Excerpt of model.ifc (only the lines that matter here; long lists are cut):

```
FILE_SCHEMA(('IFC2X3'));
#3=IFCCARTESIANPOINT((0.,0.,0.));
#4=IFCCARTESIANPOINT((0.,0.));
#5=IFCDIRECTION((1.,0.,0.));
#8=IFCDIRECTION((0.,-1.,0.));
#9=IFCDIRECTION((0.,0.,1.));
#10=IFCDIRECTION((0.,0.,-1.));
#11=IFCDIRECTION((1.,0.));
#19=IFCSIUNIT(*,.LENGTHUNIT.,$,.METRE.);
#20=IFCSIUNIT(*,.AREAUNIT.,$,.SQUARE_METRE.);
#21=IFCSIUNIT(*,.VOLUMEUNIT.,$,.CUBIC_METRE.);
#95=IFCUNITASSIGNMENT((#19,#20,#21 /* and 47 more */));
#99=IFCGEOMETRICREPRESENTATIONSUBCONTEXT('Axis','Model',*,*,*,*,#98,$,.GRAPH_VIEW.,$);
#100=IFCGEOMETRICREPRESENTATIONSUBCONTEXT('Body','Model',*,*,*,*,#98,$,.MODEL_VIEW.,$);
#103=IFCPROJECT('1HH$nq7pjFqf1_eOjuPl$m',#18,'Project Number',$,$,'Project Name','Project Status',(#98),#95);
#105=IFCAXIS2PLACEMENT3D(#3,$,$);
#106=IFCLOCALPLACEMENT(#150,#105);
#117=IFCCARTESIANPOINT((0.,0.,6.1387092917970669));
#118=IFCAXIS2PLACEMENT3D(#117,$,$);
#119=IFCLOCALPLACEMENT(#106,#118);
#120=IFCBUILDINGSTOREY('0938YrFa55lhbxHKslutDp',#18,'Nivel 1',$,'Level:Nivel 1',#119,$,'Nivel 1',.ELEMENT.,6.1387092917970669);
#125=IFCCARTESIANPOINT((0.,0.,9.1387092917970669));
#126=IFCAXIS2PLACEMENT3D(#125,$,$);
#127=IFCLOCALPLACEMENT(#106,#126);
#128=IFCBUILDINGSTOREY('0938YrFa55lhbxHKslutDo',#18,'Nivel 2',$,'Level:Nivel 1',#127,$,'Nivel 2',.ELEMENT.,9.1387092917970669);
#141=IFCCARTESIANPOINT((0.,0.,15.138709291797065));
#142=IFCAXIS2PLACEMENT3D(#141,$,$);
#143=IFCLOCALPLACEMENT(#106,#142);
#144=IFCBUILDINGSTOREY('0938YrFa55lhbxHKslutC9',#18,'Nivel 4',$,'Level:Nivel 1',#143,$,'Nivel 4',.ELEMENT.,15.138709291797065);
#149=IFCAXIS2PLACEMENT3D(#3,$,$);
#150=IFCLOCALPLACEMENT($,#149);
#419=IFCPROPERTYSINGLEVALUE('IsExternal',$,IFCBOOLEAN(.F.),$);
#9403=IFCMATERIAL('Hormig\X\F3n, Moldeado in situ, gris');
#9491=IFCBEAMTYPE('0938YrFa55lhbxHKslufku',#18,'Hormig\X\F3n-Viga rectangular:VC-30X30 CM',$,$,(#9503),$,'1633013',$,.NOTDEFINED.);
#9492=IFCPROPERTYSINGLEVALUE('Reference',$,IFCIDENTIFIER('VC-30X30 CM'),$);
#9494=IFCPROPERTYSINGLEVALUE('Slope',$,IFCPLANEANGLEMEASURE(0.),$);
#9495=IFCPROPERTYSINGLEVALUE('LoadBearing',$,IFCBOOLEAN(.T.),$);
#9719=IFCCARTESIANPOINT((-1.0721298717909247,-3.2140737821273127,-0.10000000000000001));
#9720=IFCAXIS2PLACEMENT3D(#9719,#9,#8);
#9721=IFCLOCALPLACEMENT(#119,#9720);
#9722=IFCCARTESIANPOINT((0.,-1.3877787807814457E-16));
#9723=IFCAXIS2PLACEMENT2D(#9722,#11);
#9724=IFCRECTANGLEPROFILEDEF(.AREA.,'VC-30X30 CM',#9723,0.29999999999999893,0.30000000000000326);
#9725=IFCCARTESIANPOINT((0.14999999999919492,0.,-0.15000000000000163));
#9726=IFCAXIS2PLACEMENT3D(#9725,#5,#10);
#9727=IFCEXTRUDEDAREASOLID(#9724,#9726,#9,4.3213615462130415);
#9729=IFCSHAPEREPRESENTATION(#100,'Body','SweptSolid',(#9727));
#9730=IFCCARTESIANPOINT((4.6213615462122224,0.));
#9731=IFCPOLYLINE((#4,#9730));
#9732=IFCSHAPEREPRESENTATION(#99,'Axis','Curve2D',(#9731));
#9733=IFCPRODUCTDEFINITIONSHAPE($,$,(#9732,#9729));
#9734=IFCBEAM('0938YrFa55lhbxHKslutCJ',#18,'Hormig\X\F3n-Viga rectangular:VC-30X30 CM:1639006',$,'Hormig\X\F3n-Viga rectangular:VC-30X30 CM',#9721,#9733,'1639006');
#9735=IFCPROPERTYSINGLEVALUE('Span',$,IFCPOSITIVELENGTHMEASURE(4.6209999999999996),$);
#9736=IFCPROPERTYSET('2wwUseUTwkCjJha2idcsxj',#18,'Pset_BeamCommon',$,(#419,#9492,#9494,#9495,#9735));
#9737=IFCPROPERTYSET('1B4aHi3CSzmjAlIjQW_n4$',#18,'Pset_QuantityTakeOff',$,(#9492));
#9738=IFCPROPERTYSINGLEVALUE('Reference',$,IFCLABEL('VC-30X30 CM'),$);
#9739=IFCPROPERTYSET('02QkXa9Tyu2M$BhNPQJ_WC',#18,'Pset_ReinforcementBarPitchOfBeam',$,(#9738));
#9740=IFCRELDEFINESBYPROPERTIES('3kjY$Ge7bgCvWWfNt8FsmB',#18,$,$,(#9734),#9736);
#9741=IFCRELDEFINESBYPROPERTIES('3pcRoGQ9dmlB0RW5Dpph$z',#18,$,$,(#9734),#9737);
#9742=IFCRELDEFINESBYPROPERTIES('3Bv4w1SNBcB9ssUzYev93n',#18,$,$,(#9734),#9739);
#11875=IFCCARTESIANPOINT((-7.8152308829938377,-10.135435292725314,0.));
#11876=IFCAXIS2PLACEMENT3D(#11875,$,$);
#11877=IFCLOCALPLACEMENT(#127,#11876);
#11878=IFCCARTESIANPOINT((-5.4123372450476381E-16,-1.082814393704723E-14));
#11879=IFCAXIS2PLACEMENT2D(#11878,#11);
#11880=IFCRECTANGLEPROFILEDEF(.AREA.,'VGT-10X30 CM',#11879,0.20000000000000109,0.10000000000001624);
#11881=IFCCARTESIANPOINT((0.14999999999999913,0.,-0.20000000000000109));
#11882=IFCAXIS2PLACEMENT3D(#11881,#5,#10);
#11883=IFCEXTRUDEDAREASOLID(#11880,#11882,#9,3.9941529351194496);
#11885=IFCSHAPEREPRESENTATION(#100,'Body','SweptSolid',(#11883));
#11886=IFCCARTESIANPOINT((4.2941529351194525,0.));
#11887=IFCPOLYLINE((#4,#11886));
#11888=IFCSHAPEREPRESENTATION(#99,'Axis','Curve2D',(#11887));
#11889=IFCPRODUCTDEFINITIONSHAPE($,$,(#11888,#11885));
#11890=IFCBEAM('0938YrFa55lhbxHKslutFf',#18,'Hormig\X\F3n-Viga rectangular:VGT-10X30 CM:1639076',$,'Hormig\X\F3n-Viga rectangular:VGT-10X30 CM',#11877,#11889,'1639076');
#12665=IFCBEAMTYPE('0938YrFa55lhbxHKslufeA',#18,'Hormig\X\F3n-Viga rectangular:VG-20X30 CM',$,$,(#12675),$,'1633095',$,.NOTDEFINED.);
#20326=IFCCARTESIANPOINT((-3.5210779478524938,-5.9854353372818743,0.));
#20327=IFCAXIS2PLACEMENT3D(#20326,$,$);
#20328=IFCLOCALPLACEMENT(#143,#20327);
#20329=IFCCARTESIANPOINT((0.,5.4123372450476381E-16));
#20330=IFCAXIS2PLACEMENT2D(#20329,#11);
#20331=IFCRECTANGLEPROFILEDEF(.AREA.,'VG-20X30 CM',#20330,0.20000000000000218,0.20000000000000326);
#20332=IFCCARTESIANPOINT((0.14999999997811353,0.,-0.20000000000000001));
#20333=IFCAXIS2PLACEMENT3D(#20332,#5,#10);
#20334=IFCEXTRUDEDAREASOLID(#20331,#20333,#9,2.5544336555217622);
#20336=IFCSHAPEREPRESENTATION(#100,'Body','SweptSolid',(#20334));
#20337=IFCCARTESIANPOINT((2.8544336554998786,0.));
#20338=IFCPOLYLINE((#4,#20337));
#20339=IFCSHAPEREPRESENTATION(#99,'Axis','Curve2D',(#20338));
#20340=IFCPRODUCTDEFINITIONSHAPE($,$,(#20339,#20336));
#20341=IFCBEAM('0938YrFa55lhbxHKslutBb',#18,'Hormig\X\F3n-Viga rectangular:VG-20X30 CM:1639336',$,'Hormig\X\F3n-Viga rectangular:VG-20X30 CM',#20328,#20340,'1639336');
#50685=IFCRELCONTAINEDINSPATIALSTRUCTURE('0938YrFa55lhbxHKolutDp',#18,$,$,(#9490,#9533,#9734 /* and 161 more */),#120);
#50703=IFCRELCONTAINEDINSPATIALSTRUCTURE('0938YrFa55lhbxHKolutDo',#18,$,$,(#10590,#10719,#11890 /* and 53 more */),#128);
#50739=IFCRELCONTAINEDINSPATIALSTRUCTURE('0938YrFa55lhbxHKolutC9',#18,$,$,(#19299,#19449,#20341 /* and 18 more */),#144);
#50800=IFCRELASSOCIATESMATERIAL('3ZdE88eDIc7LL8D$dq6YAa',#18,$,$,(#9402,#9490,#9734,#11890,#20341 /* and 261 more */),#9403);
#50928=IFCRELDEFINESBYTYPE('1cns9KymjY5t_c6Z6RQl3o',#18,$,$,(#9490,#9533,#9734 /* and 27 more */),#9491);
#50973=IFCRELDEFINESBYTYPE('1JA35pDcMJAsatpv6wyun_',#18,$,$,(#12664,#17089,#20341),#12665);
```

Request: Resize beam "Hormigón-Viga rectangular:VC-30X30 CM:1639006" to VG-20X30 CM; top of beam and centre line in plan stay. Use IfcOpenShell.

```python
import ifcopenshell
import ifcopenshell.api.pset
import ifcopenshell.api.type
import ifcopenshell.util.element
import ifcopenshell.util.representation

model = ifcopenshell.open("model.ifc")

member = model.by_guid("0938YrFa55lhbxHKslutCJ")
source = next(p for p in model.by_type("IfcRectangleProfileDef") if p.ProfileName == "VG-20X30 CM")

body = ifcopenshell.util.representation.get_representation(member, "Model", "Body")
solid = body.Items[0]
old_profile = solid.SweptArea

# Copy the section's sizes but keep this member's own profile position.
profile = ifcopenshell.util.element.copy(model, source)
# Profiles are centred, so shift by half the change in depth to hold the top.
shift = (old_profile.XDim - profile.XDim) / 2
x, y = old_profile.Position.Location.Coordinates
up = (-1.0, 0.0)  # upwards, in the solid's own plane
location = model.createIfcCartesianPoint((x + up[0] * shift, y + up[1] * shift))
profile.Position = model.createIfcAxis2Placement2D(location, old_profile.Position.RefDirection)
solid.SweptArea = profile
if not model.get_total_inverses(old_profile):
    ifcopenshell.util.element.remove_deep2(model, old_profile)

new_type = model.by_guid("0938YrFa55lhbxHKslufeA")
ifcopenshell.api.type.assign_type(
    model, related_objects=[member], relating_type=new_type, should_map_representations=False
)
member.Name = member.Name.replace("VC-30X30 CM", "VG-20X30 CM")
member.ObjectType = "Hormigón-Viga rectangular:VG-20X30 CM"
pset = model.by_id(ifcopenshell.util.element.get_pset(member, "Pset_BeamCommon", should_inherit=False)["id"])
ifcopenshell.api.pset.edit_pset(model, pset=pset, properties={"Reference": "VG-20X30 CM"})
pset = model.by_id(ifcopenshell.util.element.get_pset(member, "Pset_QuantityTakeOff", should_inherit=False)["id"])
ifcopenshell.api.pset.edit_pset(model, pset=pset, properties={"Reference": "VG-20X30 CM"})
pset = model.by_id(ifcopenshell.util.element.get_pset(member, "Pset_ReinforcementBarPitchOfBeam", should_inherit=False)["id"])
ifcopenshell.api.pset.edit_pset(model, pset=pset, properties={"Reference": "VG-20X30 CM"})

print(solid.SweptArea)

model.write("model_updated.ifc")
```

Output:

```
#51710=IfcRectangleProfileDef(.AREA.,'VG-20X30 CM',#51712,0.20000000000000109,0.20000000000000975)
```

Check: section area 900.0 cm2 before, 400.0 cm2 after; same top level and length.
